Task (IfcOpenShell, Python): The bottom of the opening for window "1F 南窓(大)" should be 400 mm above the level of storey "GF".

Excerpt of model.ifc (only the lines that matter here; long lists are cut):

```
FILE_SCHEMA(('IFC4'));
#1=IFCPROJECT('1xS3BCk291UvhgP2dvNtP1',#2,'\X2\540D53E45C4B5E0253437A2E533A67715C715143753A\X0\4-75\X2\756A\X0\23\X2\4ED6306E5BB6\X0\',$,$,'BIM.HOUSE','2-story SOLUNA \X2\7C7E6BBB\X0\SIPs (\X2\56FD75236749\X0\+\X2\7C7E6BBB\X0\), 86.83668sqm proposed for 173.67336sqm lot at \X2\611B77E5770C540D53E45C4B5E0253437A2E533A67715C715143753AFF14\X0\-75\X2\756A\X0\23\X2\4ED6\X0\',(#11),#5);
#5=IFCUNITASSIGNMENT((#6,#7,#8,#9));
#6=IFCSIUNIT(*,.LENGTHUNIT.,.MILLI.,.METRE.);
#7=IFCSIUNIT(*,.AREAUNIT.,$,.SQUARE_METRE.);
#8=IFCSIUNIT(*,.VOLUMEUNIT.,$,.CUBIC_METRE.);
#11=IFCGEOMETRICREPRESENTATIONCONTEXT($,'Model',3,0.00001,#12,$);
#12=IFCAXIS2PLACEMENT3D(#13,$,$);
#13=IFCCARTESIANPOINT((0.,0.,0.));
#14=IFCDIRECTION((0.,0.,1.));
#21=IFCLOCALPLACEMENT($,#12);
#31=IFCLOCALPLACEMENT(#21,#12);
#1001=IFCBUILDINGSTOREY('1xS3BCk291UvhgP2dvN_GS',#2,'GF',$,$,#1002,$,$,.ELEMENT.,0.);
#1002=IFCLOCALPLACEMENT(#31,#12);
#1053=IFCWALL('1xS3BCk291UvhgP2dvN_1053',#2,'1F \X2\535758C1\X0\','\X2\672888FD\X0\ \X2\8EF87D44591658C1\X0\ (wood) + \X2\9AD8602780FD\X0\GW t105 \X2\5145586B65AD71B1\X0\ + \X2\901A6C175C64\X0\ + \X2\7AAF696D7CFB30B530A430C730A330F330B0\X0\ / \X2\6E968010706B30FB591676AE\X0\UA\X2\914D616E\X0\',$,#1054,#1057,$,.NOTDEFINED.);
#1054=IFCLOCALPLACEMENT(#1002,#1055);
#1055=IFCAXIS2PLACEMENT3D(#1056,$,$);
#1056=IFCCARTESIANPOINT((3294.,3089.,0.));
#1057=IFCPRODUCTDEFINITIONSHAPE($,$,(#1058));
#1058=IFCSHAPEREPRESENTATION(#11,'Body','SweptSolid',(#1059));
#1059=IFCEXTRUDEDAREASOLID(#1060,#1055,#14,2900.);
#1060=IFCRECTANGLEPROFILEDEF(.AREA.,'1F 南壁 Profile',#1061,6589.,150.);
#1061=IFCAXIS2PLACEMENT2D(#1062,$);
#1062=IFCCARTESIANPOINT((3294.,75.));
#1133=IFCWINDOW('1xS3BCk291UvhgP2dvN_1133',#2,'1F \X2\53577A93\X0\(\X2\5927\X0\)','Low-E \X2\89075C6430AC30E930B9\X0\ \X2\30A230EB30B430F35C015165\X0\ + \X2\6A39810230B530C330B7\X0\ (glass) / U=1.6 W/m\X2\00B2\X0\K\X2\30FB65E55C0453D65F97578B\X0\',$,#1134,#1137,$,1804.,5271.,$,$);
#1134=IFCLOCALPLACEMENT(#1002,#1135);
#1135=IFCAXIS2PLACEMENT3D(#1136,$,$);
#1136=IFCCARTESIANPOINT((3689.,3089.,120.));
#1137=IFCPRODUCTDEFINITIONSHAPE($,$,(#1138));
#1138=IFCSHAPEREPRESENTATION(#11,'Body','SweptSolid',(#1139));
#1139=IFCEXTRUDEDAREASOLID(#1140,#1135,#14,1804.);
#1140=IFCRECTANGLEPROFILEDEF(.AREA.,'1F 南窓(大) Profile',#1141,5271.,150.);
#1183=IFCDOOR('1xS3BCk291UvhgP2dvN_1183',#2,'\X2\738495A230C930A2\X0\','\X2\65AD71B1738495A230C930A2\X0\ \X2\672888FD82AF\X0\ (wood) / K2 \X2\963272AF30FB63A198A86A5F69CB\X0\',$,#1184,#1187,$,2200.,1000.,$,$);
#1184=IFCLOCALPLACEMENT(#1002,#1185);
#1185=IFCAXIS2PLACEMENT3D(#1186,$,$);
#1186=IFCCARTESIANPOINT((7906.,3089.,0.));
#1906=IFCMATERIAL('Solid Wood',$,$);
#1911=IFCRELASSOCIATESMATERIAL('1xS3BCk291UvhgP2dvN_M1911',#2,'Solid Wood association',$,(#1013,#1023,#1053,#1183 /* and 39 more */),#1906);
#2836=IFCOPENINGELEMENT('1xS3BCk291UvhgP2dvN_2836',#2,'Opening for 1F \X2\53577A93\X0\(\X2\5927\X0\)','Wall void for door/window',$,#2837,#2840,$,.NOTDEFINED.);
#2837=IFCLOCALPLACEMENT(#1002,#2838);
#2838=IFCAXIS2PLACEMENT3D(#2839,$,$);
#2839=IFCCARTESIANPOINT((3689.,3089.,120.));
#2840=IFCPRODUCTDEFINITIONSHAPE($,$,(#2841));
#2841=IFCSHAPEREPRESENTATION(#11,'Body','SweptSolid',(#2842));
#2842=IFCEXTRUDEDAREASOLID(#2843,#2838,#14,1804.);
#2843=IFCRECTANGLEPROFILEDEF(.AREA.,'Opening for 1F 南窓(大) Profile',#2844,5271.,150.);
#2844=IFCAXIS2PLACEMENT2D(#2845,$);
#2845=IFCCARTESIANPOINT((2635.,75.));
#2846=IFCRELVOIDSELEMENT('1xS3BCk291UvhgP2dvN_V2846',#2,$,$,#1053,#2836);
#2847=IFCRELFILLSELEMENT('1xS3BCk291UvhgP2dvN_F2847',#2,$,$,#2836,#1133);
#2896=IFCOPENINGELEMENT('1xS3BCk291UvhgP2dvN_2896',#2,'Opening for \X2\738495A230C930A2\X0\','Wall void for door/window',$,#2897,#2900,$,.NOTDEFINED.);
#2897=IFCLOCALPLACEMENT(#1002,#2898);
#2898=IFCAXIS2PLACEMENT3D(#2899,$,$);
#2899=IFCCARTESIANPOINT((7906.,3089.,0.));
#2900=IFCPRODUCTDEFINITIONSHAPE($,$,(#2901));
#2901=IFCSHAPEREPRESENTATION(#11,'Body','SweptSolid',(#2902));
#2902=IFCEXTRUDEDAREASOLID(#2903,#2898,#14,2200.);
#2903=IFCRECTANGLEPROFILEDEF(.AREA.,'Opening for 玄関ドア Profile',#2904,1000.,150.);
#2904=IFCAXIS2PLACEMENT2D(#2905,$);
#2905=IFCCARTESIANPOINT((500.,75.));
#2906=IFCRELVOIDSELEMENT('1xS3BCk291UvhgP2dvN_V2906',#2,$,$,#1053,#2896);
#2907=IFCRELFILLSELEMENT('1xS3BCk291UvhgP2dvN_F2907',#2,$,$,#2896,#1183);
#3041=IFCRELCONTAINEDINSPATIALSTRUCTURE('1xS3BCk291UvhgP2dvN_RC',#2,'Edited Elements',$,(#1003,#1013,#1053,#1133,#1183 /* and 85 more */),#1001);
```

```python
import numpy as np
import ifcopenshell
import ifcopenshell.api.geometry
import ifcopenshell.geom
import ifcopenshell.util.element
import ifcopenshell.util.placement
import ifcopenshell.util.shape
import ifcopenshell.util.unit

model = ifcopenshell.open("model.ifc")
unit_scale = ifcopenshell.util.unit.calculate_unit_scale(model)

window = model.by_id(1133)
opening = window.FillsVoids[0].RelatingOpeningElement
storey = ifcopenshell.util.element.get_container(window, ifc_class="IfcBuildingStorey")
level = ifcopenshell.util.placement.get_local_placement(storey.ObjectPlacement)[2, 3]

# The opening's origin need not be at the sill, so measure its lowest point.
shape = ifcopenshell.geom.create_shape(ifcopenshell.geom.settings(), opening)
bottom = ifcopenshell.util.shape.get_shape_bottom_elevation(shape, shape.geometry) / unit_scale
dz = level + 400.0 - bottom

shift = np.array([0.0, 0.0, dz])
# The window is not placed relative to its opening, so move both.
for product in (opening, window):
    matrix = ifcopenshell.util.placement.get_local_placement(product.ObjectPlacement)
    matrix[:3, 3] += shift
    ifcopenshell.api.geometry.edit_object_placement(model, product=product, matrix=matrix, is_si=False)

print(f"moved by {dz * unit_scale:+.3f} m")

model.write("model-out.ifc")
```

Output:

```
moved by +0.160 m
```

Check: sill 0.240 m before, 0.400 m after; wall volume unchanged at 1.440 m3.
